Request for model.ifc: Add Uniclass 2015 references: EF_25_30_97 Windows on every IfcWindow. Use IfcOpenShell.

First a look at what the model holds.

```python
import ifcopenshell

model = ifcopenshell.open("model.ifc")
print(model.schema)
print("classifications:", [c.Name for c in model.by_type("IfcClassification")])
for ifc_class in ("IfcDoor", "IfcRoof", "IfcStair", "IfcWall", "IfcWindow"):
    print(ifc_class, len(model.by_type(ifc_class)))
```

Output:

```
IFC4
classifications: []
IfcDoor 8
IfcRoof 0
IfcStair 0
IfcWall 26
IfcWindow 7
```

```python
import ifcopenshell
import ifcopenshell.api.classification

model = ifcopenshell.open("model.ifc")

system = ifcopenshell.api.classification.add_classification(model, classification="Uniclass 2015")

codes = {
    "IfcWindow": ("EF_25_30_97", "Windows"),
}
for ifc_class, (code, name) in codes.items():
    products = model.by_type(ifc_class)
    ifcopenshell.api.classification.add_reference(
        model, products=products, classification=system, identification=code, name=name
    )
    print(code, len(products))

model.write("model-out.ifc")
```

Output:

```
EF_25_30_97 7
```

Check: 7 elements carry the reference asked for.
